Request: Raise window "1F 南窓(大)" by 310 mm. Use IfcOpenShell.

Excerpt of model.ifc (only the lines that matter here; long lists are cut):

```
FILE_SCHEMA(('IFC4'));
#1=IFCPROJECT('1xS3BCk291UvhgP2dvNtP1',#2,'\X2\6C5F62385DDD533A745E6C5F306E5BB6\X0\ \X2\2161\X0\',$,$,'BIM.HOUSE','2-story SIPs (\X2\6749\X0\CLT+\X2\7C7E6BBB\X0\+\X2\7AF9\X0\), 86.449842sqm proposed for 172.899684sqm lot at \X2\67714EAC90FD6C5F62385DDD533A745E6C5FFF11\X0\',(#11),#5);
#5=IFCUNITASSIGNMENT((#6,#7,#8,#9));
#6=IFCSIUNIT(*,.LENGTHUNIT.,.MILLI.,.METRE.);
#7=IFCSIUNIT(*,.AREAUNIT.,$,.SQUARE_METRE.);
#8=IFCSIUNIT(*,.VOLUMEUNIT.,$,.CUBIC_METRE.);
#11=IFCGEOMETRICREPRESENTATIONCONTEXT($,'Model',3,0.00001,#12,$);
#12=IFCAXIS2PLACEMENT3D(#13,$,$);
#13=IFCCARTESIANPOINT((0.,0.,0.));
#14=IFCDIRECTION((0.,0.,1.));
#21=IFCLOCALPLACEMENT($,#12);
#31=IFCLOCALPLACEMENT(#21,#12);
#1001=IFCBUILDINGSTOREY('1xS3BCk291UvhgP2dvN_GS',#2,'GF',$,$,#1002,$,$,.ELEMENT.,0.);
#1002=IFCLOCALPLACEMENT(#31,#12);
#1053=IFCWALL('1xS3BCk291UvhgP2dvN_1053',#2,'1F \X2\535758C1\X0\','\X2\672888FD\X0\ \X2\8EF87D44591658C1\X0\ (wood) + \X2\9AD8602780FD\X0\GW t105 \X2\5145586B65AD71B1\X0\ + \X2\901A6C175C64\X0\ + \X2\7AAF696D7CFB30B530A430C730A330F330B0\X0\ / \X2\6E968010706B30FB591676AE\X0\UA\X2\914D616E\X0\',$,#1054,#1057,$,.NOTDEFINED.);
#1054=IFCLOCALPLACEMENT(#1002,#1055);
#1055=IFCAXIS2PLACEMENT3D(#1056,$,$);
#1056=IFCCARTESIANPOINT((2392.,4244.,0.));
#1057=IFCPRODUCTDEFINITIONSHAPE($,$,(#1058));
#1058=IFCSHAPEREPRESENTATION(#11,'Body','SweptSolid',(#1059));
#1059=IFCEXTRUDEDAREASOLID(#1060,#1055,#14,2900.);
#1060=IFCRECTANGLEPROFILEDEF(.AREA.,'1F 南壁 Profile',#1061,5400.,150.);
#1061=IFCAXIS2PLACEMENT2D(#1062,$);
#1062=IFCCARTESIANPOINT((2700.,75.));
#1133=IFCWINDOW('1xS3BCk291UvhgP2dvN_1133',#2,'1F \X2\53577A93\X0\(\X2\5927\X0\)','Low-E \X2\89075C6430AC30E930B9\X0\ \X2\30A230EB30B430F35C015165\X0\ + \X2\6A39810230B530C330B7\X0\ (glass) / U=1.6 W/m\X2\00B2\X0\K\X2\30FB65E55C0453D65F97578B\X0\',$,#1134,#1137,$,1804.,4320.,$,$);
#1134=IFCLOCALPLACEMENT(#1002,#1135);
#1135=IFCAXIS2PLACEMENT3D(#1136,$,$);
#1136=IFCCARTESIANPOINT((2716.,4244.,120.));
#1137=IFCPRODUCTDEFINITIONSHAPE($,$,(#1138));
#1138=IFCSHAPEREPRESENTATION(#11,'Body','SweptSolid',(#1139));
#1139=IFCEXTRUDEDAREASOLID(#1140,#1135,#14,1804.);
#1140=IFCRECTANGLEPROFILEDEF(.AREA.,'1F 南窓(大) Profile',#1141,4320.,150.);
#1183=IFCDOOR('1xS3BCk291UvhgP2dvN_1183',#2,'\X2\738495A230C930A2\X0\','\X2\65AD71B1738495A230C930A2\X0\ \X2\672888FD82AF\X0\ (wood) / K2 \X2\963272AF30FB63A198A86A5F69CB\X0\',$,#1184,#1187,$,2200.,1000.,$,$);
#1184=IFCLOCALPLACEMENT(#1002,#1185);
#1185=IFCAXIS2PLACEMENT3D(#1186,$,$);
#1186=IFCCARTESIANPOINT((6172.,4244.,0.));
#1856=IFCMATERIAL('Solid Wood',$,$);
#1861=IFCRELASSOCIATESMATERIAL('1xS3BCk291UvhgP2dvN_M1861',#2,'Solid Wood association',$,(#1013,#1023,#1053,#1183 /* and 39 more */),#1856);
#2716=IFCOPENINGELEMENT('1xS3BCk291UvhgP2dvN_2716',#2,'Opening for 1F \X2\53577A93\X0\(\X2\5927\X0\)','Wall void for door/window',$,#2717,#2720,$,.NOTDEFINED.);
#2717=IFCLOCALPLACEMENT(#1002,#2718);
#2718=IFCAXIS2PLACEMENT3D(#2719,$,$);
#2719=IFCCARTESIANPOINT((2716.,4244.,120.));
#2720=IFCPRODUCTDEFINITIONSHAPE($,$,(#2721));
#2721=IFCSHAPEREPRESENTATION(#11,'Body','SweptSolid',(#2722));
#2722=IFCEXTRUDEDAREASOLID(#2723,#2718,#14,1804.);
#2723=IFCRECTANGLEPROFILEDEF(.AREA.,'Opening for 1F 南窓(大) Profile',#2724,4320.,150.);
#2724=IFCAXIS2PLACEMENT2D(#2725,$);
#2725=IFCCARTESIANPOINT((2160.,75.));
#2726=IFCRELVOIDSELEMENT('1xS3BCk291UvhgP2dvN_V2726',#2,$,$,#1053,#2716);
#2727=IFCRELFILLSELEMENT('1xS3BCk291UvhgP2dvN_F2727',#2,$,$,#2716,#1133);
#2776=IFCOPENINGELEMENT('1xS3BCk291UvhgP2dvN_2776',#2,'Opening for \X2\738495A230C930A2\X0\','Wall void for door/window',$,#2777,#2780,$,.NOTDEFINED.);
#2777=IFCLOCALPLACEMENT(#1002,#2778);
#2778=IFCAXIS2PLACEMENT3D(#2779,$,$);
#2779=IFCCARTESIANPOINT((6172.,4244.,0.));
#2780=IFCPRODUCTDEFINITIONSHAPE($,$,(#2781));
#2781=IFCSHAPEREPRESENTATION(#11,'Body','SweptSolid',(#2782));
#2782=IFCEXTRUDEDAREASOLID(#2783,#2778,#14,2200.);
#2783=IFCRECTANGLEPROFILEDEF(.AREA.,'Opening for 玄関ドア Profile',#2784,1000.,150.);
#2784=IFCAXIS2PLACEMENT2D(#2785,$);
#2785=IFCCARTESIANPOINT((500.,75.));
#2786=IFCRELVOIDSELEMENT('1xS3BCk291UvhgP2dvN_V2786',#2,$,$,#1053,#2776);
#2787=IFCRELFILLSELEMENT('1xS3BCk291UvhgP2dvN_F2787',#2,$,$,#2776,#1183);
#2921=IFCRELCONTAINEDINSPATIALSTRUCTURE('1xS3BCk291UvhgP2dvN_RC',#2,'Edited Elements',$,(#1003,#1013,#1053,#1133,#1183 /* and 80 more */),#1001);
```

```python
import numpy as np
import ifcopenshell
import ifcopenshell.api.geometry
import ifcopenshell.util.placement
import ifcopenshell.util.unit

model = ifcopenshell.open("model.ifc")
unit_scale = ifcopenshell.util.unit.calculate_unit_scale(model)

window = model.by_id(1133)
opening = window.FillsVoids[0].RelatingOpeningElement
dz = 0.31 / unit_scale

shift = np.array([0.0, 0.0, dz])
# The window is not placed relative to its opening, so move both.
for product in (opening, window):
    matrix = ifcopenshell.util.placement.get_local_placement(product.ObjectPlacement)
    matrix[:3, 3] += shift
    ifcopenshell.api.geometry.edit_object_placement(model, product=product, matrix=matrix, is_si=False)

print(f"moved by {dz * unit_scale:+.3f} m")

model.write("model_rev.ifc")
```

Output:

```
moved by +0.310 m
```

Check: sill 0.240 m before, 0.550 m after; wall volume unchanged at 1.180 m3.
